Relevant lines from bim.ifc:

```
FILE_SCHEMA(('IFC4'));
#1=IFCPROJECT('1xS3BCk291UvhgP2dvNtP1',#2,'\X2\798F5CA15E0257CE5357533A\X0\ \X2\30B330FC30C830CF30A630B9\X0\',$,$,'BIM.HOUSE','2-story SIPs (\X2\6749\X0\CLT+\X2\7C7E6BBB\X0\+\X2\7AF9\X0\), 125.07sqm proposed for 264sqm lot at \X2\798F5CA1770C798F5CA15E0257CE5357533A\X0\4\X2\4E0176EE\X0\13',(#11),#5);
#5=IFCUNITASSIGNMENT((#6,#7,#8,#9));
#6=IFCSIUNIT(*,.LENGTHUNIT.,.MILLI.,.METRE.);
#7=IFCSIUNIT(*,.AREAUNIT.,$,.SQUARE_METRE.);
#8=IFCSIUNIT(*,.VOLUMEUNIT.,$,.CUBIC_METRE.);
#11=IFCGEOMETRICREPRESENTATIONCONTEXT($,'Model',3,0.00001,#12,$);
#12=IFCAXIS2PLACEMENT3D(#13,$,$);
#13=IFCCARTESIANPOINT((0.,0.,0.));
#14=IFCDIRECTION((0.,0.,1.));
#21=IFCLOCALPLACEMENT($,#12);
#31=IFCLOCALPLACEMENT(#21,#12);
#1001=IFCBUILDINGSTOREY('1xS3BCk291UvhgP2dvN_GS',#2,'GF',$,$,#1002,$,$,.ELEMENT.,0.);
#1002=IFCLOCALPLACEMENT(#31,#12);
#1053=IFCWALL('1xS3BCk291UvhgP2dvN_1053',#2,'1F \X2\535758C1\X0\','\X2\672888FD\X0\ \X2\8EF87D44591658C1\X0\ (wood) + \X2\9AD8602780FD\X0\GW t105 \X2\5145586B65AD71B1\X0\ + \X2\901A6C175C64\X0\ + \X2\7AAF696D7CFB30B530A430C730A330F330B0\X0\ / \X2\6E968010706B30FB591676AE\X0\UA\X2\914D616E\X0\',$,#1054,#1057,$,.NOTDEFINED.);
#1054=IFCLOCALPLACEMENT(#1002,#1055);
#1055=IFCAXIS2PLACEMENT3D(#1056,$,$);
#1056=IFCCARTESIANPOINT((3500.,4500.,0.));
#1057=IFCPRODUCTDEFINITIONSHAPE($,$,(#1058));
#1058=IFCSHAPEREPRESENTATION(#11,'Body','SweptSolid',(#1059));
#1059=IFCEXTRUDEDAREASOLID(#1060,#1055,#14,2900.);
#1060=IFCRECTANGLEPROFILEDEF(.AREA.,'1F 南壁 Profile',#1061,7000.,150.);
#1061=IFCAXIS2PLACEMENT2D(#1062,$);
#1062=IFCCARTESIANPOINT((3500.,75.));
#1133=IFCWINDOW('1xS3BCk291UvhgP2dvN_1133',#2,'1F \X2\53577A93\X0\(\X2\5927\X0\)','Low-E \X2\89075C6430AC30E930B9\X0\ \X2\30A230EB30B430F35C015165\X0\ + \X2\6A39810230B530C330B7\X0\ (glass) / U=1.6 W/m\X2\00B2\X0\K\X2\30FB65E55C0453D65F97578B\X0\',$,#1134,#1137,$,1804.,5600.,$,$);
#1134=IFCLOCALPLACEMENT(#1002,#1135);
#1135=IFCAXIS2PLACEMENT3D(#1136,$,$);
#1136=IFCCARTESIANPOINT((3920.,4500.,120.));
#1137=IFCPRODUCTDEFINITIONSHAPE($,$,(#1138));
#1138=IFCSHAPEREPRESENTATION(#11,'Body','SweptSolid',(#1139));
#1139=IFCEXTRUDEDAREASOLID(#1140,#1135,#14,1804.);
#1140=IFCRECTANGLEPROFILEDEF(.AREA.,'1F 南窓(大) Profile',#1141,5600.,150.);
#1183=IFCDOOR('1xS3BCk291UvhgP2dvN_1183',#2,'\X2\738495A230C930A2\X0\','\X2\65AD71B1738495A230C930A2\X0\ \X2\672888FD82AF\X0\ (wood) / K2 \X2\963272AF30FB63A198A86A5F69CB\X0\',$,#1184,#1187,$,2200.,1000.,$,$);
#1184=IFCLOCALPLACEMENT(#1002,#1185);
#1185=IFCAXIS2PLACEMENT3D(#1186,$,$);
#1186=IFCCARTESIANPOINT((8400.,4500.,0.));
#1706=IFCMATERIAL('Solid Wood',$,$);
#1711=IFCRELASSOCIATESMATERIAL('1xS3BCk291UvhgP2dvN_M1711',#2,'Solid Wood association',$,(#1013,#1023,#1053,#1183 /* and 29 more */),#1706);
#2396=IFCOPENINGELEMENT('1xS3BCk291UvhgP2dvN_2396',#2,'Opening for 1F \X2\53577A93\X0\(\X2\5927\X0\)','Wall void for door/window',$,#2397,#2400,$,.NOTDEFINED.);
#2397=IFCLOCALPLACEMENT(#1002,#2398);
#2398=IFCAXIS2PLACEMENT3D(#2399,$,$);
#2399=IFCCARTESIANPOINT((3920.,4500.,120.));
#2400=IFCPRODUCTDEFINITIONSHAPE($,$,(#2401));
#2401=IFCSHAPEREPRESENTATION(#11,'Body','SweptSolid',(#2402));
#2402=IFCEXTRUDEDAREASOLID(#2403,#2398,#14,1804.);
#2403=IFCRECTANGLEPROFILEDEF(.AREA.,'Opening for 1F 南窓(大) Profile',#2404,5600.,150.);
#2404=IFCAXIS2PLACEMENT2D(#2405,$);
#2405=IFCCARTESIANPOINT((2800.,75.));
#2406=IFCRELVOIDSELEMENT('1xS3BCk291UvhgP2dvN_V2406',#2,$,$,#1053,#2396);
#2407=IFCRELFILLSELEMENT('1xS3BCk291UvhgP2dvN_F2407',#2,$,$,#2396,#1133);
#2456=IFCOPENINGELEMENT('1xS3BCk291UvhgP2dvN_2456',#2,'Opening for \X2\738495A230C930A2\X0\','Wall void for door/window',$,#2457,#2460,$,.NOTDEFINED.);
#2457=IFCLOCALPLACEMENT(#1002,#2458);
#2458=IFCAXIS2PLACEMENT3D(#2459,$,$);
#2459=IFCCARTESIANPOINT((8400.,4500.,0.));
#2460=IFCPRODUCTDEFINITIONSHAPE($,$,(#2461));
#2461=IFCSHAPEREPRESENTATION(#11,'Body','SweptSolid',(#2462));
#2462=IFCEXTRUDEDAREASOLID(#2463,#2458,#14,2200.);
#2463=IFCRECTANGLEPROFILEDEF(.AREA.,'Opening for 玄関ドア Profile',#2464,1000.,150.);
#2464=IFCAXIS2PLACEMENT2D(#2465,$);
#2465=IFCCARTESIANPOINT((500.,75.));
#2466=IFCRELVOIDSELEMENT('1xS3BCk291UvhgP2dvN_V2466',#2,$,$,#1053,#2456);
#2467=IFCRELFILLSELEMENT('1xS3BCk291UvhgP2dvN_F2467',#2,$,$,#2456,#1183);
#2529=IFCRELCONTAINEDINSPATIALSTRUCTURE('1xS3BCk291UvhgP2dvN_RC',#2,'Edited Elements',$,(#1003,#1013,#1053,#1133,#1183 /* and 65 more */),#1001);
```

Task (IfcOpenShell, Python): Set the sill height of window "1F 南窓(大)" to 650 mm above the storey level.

```python
import numpy as np
import ifcopenshell
import ifcopenshell.api.geometry
import ifcopenshell.geom
import ifcopenshell.util.element
import ifcopenshell.util.placement
import ifcopenshell.util.shape
import ifcopenshell.util.unit

model = ifcopenshell.open("bim.ifc")
unit_scale = ifcopenshell.util.unit.calculate_unit_scale(model)

window = model.by_guid("1xS3BCk291UvhgP2dvN_1133")
opening = window.FillsVoids[0].RelatingOpeningElement
storey = ifcopenshell.util.element.get_container(window, ifc_class="IfcBuildingStorey")
level = ifcopenshell.util.placement.get_local_placement(storey.ObjectPlacement)[2, 3]

# The opening's origin need not be at the sill, so measure its lowest point.
shape = ifcopenshell.geom.create_shape(ifcopenshell.geom.settings(), opening)
bottom = ifcopenshell.util.shape.get_shape_bottom_elevation(shape, shape.geometry) / unit_scale
dz = level + 0.65 / unit_scale - bottom

shift = np.array([0.0, 0.0, dz])
# The window is not placed relative to its opening, so move both.
for product in (opening, window):
    matrix = ifcopenshell.util.placement.get_local_placement(product.ObjectPlacement)
    matrix[:3, 3] += shift
    ifcopenshell.api.geometry.edit_object_placement(model, product=product, matrix=matrix, is_si=False)

print(f"moved by {dz * unit_scale:+.3f} m")

model.write("bim_edited.ifc")
```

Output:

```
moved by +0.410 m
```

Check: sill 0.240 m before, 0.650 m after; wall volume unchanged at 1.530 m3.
